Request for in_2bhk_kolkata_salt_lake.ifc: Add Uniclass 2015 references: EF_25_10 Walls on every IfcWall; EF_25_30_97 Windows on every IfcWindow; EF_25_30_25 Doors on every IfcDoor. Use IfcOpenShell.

First a look at what the model holds.

```python
import ifcopenshell

model = ifcopenshell.open("in_2bhk_kolkata_salt_lake.ifc")
print(model.schema)
print("classifications:", [c.Name for c in model.by_type("IfcClassification")])
for ifc_class in ("IfcDoor", "IfcRoof", "IfcStair", "IfcWall", "IfcWindow"):
    print(ifc_class, len(model.by_type(ifc_class)))
```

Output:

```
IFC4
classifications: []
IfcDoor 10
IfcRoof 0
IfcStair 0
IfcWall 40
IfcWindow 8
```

```python
import ifcopenshell
import ifcopenshell.api.classification

model = ifcopenshell.open("in_2bhk_kolkata_salt_lake.ifc")

system = ifcopenshell.api.classification.add_classification(model, classification="Uniclass 2015")

codes = {
    "IfcWall": ("EF_25_10", "Walls"),
    "IfcWindow": ("EF_25_30_97", "Windows"),
    "IfcDoor": ("EF_25_30_25", "Doors"),
}
for ifc_class, (code, name) in codes.items():
    products = model.by_type(ifc_class)
    ifcopenshell.api.classification.add_reference(
        model, products=products, classification=system, identification=code, name=name
    )
    print(code, len(products))

model.write("in_2bhk_kolkata_salt_lake_rev.ifc")
```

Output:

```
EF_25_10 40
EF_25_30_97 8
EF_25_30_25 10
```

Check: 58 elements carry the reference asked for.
